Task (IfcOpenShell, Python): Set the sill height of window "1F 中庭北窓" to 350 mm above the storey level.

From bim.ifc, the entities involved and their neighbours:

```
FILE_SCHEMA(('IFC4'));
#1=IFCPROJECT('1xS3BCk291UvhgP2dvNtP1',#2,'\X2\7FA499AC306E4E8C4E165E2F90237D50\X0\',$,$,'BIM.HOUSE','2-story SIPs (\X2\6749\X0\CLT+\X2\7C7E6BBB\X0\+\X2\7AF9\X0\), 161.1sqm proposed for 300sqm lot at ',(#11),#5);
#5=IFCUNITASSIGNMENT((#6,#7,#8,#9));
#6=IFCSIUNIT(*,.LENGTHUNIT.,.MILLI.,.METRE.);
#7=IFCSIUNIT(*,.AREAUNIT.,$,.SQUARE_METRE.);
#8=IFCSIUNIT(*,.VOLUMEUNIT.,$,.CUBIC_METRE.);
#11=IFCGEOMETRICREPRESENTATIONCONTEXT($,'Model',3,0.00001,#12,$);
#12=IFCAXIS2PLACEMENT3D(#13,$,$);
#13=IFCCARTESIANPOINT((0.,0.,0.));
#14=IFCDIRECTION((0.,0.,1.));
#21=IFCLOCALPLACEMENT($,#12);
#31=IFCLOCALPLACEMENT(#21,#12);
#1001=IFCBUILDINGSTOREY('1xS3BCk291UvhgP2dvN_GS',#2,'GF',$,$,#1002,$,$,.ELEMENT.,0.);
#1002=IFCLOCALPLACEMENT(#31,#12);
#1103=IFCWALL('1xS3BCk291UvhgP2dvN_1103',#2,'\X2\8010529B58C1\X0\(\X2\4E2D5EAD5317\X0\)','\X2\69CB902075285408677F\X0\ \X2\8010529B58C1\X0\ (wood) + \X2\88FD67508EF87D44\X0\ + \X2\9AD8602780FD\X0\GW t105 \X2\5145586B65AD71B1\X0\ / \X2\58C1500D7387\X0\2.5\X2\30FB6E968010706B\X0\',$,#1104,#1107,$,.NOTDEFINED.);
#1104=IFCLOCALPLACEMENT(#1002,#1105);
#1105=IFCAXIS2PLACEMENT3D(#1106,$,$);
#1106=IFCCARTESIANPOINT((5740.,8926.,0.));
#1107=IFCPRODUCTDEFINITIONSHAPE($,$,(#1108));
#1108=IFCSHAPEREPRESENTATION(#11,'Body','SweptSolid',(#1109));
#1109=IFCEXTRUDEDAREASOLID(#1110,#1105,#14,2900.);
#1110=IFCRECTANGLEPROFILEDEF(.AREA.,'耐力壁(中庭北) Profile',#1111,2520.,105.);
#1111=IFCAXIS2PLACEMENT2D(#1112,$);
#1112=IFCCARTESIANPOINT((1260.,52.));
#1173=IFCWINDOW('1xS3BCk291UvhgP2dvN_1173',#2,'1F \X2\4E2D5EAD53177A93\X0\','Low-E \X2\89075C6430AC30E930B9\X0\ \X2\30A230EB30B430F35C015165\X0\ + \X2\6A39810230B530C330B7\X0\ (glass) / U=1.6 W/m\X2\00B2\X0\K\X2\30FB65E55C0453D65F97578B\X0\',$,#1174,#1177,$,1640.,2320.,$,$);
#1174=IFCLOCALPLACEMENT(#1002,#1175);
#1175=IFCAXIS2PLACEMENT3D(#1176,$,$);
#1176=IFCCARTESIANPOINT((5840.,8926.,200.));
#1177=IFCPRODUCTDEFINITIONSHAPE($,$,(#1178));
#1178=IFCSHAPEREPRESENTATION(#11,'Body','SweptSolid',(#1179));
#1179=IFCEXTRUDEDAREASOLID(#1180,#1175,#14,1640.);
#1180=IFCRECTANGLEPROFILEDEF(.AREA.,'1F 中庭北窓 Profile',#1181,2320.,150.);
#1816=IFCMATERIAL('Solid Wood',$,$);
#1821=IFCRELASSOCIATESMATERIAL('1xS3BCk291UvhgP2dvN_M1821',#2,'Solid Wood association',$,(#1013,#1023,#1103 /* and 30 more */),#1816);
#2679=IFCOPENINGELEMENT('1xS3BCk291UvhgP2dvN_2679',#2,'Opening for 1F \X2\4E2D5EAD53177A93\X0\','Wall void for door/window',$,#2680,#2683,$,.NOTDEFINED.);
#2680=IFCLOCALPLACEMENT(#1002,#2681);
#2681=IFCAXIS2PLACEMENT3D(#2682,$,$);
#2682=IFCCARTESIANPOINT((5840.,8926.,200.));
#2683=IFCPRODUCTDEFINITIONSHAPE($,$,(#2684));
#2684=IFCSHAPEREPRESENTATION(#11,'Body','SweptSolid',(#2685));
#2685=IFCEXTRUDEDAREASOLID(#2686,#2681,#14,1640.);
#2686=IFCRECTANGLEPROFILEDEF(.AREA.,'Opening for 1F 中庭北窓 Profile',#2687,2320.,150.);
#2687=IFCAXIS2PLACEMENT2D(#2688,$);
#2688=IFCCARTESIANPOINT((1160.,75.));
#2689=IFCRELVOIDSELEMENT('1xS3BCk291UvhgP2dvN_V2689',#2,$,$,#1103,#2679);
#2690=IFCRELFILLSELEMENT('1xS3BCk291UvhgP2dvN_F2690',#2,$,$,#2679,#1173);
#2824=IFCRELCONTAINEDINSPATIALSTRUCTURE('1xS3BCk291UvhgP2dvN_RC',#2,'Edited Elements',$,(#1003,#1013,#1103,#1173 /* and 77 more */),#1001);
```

```python
import numpy as np
import ifcopenshell
import ifcopenshell.api.geometry
import ifcopenshell.geom
import ifcopenshell.util.element
import ifcopenshell.util.placement
import ifcopenshell.util.shape
import ifcopenshell.util.unit

model = ifcopenshell.open("bim.ifc")
unit_scale = ifcopenshell.util.unit.calculate_unit_scale(model)

window = model.by_guid("1xS3BCk291UvhgP2dvN_1173")
opening = window.FillsVoids[0].RelatingOpeningElement
storey = ifcopenshell.util.element.get_container(window, ifc_class="IfcBuildingStorey")
level = ifcopenshell.util.placement.get_local_placement(storey.ObjectPlacement)[2, 3]

# The opening's origin need not be at the sill, so measure its lowest point.
shape = ifcopenshell.geom.create_shape(ifcopenshell.geom.settings(), opening)
bottom = ifcopenshell.util.shape.get_shape_bottom_elevation(shape, shape.geometry) / unit_scale
dz = level + 0.35 / unit_scale - bottom

shift = np.array([0.0, 0.0, dz])
# The window is not placed relative to its opening, so move both.
for product in (opening, window):
    matrix = ifcopenshell.util.placement.get_local_placement(product.ObjectPlacement)
    matrix[:3, 3] += shift
    ifcopenshell.api.geometry.edit_object_placement(model, product=product, matrix=matrix, is_si=False)

print(f"moved by {dz * unit_scale:+.3f} m")

model.write("bim_rev.ifc")
```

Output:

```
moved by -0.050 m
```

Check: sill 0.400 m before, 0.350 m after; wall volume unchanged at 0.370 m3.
